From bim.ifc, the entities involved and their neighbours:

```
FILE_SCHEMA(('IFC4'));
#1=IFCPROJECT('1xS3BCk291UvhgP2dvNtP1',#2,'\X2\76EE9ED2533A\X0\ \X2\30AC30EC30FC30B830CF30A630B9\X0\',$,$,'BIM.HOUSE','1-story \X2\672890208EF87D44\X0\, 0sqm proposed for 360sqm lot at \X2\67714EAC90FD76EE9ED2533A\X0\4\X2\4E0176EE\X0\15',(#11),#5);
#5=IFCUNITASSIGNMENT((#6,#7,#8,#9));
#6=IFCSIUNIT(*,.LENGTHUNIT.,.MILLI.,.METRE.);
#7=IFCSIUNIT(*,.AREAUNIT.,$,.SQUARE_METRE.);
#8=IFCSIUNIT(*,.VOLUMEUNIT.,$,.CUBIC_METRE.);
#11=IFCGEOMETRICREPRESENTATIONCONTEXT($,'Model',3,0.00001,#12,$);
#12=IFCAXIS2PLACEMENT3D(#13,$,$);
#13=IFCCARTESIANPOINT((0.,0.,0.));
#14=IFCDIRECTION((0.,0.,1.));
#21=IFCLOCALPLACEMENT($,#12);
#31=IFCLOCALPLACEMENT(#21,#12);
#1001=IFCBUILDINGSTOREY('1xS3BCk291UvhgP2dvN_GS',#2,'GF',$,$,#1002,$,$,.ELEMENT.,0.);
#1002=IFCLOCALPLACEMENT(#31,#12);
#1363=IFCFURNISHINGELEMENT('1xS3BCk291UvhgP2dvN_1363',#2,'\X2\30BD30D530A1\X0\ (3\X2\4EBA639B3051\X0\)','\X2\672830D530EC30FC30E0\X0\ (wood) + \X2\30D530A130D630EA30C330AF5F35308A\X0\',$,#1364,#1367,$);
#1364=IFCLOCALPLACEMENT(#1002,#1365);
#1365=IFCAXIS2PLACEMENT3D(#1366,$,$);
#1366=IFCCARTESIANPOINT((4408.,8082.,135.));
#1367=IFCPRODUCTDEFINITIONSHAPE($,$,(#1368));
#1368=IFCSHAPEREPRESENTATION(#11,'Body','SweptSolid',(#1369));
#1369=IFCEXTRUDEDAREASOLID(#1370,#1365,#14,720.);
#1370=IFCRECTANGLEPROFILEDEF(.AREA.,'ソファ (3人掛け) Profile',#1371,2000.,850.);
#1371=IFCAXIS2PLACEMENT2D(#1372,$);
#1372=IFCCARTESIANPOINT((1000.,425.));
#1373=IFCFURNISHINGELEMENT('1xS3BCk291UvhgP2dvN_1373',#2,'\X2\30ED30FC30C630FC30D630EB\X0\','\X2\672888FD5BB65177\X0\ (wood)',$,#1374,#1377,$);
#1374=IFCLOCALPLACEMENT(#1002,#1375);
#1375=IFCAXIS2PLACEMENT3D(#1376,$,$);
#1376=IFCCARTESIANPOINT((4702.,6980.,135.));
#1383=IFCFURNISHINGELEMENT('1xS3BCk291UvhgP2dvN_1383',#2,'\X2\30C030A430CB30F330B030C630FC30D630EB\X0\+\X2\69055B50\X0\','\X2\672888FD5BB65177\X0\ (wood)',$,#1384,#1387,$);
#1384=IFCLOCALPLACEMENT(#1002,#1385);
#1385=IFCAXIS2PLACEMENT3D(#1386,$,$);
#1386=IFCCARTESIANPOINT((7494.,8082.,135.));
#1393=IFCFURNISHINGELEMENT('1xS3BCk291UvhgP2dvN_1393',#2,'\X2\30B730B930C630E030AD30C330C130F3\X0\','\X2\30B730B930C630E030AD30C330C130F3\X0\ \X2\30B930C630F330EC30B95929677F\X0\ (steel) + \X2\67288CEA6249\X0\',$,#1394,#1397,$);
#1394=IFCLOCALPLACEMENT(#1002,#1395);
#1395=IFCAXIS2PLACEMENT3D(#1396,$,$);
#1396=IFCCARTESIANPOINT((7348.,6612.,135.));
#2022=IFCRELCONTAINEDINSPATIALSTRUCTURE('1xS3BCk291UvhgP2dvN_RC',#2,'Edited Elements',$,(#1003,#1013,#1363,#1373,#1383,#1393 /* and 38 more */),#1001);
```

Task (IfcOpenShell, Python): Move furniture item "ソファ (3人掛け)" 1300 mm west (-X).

```python
import ifcopenshell
import ifcopenshell.api.geometry
import ifcopenshell.util.placement

model = ifcopenshell.open("bim.ifc")

item = model.by_guid("1xS3BCk291UvhgP2dvN_1363")
matrix = ifcopenshell.util.placement.get_local_placement(item.ObjectPlacement)
matrix[0, 3] -= 1300.0
ifcopenshell.api.geometry.edit_object_placement(model, product=item, matrix=matrix, is_si=False)

print(ifcopenshell.util.placement.get_local_placement(item.ObjectPlacement).round(3) + 0.0)

model.write("bim_v2.ifc")
```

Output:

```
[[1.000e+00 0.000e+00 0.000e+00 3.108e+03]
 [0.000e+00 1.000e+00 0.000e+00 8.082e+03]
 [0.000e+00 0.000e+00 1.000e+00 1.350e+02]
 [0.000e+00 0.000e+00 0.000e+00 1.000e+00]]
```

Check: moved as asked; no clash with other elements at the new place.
